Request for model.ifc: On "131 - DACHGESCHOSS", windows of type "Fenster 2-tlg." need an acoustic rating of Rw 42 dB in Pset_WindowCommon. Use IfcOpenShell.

First a look at what the model holds.

```python
import ifcopenshell
import ifcopenshell.util.element

model = ifcopenshell.open("model.ifc")
print(model.schema)
storey = next(s for s in model.by_type("IfcBuildingStorey") if s.Name == "131 - DACHGESCHOSS")
windows = [e for e in ifcopenshell.util.element.get_decomposition(storey) if e.is_a("IfcWindow")]
seen = {}
for e in windows:
    element_type = ifcopenshell.util.element.get_type(e)
    key = (element_type.Name if element_type != e and element_type else None, ifcopenshell.util.element.get_pset(e, "Pset_WindowCommon", "AcousticRating"))
    seen[key] = seen.get(key, 0) + 1
for (name, value), count in sorted(seen.items(), key=str):
    print(count, "x", name, "|", value)
```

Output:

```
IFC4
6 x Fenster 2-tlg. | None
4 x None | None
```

```python
import ifcopenshell
import ifcopenshell.api.pset
import ifcopenshell.util.element

model = ifcopenshell.open("model.ifc")

storey = next(s for s in model.by_type("IfcBuildingStorey") if s.Name == "131 - DACHGESCHOSS")
windows = [e for e in ifcopenshell.util.element.get_decomposition(storey) if e.is_a("IfcWindow")]

count = 0
for e in windows:
    element_type = ifcopenshell.util.element.get_type(e)
    if element_type in (None, e) or element_type.Name != "Fenster 2-tlg.":
        continue
    # add_pset returns the element's existing set when there is one.
    pset = ifcopenshell.api.pset.add_pset(model, product=e, name="Pset_WindowCommon")
    ifcopenshell.api.pset.edit_pset(model, pset=pset, properties={"AcousticRating": "Rw 42 dB"})
    count += 1

print(count, "windows updated")

model.write("model_rev.ifc")
```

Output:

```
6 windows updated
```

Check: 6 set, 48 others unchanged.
